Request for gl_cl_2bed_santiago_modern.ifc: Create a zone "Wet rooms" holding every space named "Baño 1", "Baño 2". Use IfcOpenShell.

First a look at what the model holds.

```python
import ifcopenshell

model = ifcopenshell.open("gl_cl_2bed_santiago_modern.ifc")
print(model.schema)
seen = {}
for space in model.by_type("IfcSpace"):
    seen[space.LongName] = seen.get(space.LongName, 0) + 1
for name, count in sorted(seen.items(), key=str):
    print(count, "x", name)
print("zones:", [z.Name for z in model.by_type("IfcZone")][:20])
```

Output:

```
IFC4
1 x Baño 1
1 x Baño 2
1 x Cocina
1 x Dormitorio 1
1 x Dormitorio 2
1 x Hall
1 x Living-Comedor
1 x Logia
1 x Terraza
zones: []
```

```python
import ifcopenshell
import ifcopenshell.api.group
import ifcopenshell.api.root

model = ifcopenshell.open("gl_cl_2bed_santiago_modern.ifc")

names = {"Baño 1", "Baño 2"}
spaces = [s for s in model.by_type("IfcSpace") if s.LongName in names]

zone = ifcopenshell.api.root.create_entity(model, ifc_class="IfcZone", name="Wet rooms")
ifcopenshell.api.group.assign_group(model, products=spaces, group=zone)
print(len(spaces), "spaces in", zone.Name)

model.write("gl_cl_2bed_santiago_modern-out.ifc")
```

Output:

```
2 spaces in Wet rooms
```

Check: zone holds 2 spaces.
